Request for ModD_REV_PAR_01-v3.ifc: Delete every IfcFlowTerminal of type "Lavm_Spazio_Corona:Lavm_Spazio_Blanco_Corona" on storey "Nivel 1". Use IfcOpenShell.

First a look at what the model holds.

```python
import ifcopenshell
import ifcopenshell.util.element

model = ifcopenshell.open("ModD_REV_PAR_01-v3.ifc")
print(model.schema)
storey = next(s for s in model.by_type("IfcBuildingStorey") if s.Name == "Nivel 1")
terminals = [e for e in ifcopenshell.util.element.get_decomposition(storey) if e.is_a("IfcFlowTerminal")]
seen = {}
for e in terminals:
    element_type = ifcopenshell.util.element.get_type(e)
    name = element_type.Name if element_type not in (None, e) else None
    seen[name] = seen.get(name, 0) + 1
for name, count in sorted(seen.items(), key=str):
    print(count, "x", name)
```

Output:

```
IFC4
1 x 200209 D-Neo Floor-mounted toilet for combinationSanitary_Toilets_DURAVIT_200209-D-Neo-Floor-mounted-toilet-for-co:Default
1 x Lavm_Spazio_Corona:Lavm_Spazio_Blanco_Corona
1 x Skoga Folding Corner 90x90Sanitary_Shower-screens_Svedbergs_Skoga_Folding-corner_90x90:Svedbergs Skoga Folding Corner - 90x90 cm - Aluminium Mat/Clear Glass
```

```python
import ifcopenshell
import ifcopenshell.api.root
import ifcopenshell.util.element

model = ifcopenshell.open("ModD_REV_PAR_01-v3.ifc")

storey = next(s for s in model.by_type("IfcBuildingStorey") if s.Name == "Nivel 1")
terminals = [e for e in ifcopenshell.util.element.get_decomposition(storey) if e.is_a("IfcFlowTerminal")]
targets = [e for e in terminals if (t := ifcopenshell.util.element.get_type(e)) not in (None, e) and t.Name == "Lavm_Spazio_Corona:Lavm_Spazio_Blanco_Corona"]

for e in targets:
    ifcopenshell.api.root.remove_product(model, product=e)
print(len(targets), "removed")

model.write("ModD_REV_PAR_01-v3-out.ifc")
```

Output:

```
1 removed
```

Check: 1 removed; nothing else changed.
